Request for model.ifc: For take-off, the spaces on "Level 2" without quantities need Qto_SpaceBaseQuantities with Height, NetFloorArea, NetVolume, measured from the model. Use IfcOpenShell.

First a look at what the model holds.

```python
import ifcopenshell
import ifcopenshell.util.element
import ifcopenshell.util.unit

model = ifcopenshell.open("model.ifc")
print(model.schema)
for unit_type in ("LENGTHUNIT", "AREAUNIT", "VOLUMEUNIT"):
    print(unit_type, ifcopenshell.util.unit.calculate_unit_scale(model, unit_type))
storey = next(s for s in model.by_type("IfcBuildingStorey") if s.Name == "Level 2")
spaces = [e for e in ifcopenshell.util.element.get_decomposition(storey) if e.is_a("IfcSpace")]
for e in sorted(spaces, key=lambda e: e.id()):
    print(e.id(), e.is_a(), e.Name, list(ifcopenshell.util.element.get_psets(e, qtos_only=True)), sep=" | ")
```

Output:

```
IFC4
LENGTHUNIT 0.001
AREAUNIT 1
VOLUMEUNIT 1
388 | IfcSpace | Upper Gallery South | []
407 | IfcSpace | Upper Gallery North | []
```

```python
import ifcopenshell
import ifcopenshell.api.pset
import ifcopenshell.geom
import ifcopenshell.util.element
import ifcopenshell.util.shape
import ifcopenshell.util.unit

model = ifcopenshell.open("model.ifc")
unit_scale = ifcopenshell.util.unit.calculate_unit_scale(model)
area_scale = ifcopenshell.util.unit.calculate_unit_scale(model, "AREAUNIT")
volume_scale = ifcopenshell.util.unit.calculate_unit_scale(model, "VOLUMEUNIT")
settings = ifcopenshell.geom.settings()

storey = next(s for s in model.by_type("IfcBuildingStorey") if s.Name == "Level 2")
spaces = [e for e in ifcopenshell.util.element.get_decomposition(storey) if e.is_a("IfcSpace")]

for e in sorted(spaces, key=lambda e: e.id()):
    if ifcopenshell.util.element.get_psets(e, qtos_only=True, should_inherit=False):
        continue
    # Geometry comes back in metres, in the element's own axes.
    shape = ifcopenshell.geom.create_shape(settings, e)
    values = {
        "Height": ifcopenshell.util.shape.get_z(shape.geometry) / unit_scale,
        "NetFloorArea": ifcopenshell.util.shape.get_footprint_area(shape.geometry) / area_scale,
        "NetVolume": ifcopenshell.util.shape.get_volume(shape.geometry) / volume_scale,
    }
    qto = ifcopenshell.api.pset.add_qto(model, product=e, name="Qto_SpaceBaseQuantities")
    ifcopenshell.api.pset.edit_qto(model, qto=qto, properties=values)
    print(e.id(), {k: round(v, 3) for k, v in values.items()})

model.write("model_v2.ifc")
```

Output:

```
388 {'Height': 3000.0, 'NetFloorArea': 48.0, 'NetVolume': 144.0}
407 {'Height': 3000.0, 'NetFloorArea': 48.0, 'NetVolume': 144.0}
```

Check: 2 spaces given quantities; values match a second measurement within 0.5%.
